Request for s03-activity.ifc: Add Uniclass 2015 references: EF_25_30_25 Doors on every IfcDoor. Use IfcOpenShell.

First a look at what the model holds.

```python
import ifcopenshell

model = ifcopenshell.open("s03-activity.ifc")
print(model.schema)
print("classifications:", [c.Name for c in model.by_type("IfcClassification")])
for ifc_class in ("IfcDoor", "IfcRoof", "IfcStair", "IfcWall", "IfcWindow"):
    print(ifc_class, len(model.by_type(ifc_class)))
```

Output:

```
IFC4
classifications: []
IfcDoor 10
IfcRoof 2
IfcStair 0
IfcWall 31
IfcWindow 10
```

```python
import ifcopenshell
import ifcopenshell.api.classification

model = ifcopenshell.open("s03-activity.ifc")

system = ifcopenshell.api.classification.add_classification(model, classification="Uniclass 2015")

codes = {
    "IfcDoor": ("EF_25_30_25", "Doors"),
}
for ifc_class, (code, name) in codes.items():
    products = model.by_type(ifc_class)
    ifcopenshell.api.classification.add_reference(
        model, products=products, classification=system, identification=code, name=name
    )
    print(code, len(products))

model.write("s03-activity_updated.ifc")
```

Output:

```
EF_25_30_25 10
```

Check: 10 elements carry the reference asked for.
